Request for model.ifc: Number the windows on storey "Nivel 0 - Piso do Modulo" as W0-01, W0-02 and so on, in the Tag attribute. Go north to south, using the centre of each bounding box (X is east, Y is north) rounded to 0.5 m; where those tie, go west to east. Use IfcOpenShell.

First a look at what the model holds.

```python
import ifcopenshell
import ifcopenshell.util.element
import ifcopenshell.util.placement

model = ifcopenshell.open("model.ifc")
print(model.schema)
storey = next(s for s in model.by_type("IfcBuildingStorey") if s.Name == "Nivel 0 - Piso do Modulo")
windows = [e for e in ifcopenshell.util.element.get_decomposition(storey) if e.is_a("IfcWindow")]
for e in sorted(windows, key=lambda e: e.id()):
    origin = ifcopenshell.util.placement.get_local_placement(e.ObjectPlacement)[:3, 3]
    print(e.id(), e.Tag, e.Name, origin.round(2) + 0.0, sep=" | ")
```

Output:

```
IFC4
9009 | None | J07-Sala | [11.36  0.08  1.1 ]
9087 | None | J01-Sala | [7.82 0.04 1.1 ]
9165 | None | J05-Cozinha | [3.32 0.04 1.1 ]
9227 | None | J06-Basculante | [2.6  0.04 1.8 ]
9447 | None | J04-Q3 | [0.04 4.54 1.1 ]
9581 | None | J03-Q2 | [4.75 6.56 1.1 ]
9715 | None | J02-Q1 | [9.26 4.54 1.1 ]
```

```python
import ifcopenshell
import ifcopenshell.geom
import ifcopenshell.util.element
import ifcopenshell.util.shape

model = ifcopenshell.open("model.ifc")
settings = ifcopenshell.geom.settings()
settings.set("use-world-coords", True)


def centre(element):
    shape = ifcopenshell.geom.create_shape(settings, element)
    return ifcopenshell.util.shape.get_bbox_centroid(shape.geometry)


storey = next(s for s in model.by_type("IfcBuildingStorey") if s.Name == "Nivel 0 - Piso do Modulo")
windows = [e for e in ifcopenshell.util.element.get_decomposition(storey) if e.is_a("IfcWindow")]

# Insertion points can sit at a corner or the storey origin, so sort by the geometry (in metres).
centres = {e: centre(e) for e in windows}
windows.sort(key=lambda e: (-round(centres[e][1] / 0.5), centres[e][0]))

for i, e in enumerate(windows, start=1):
    number = f"W0-{i:02d}"
    e.Tag = number
    print(e.id(), number)

model.write("model_edited.ifc")
```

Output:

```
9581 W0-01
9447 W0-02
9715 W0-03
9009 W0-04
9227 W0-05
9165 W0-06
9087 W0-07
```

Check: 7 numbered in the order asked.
